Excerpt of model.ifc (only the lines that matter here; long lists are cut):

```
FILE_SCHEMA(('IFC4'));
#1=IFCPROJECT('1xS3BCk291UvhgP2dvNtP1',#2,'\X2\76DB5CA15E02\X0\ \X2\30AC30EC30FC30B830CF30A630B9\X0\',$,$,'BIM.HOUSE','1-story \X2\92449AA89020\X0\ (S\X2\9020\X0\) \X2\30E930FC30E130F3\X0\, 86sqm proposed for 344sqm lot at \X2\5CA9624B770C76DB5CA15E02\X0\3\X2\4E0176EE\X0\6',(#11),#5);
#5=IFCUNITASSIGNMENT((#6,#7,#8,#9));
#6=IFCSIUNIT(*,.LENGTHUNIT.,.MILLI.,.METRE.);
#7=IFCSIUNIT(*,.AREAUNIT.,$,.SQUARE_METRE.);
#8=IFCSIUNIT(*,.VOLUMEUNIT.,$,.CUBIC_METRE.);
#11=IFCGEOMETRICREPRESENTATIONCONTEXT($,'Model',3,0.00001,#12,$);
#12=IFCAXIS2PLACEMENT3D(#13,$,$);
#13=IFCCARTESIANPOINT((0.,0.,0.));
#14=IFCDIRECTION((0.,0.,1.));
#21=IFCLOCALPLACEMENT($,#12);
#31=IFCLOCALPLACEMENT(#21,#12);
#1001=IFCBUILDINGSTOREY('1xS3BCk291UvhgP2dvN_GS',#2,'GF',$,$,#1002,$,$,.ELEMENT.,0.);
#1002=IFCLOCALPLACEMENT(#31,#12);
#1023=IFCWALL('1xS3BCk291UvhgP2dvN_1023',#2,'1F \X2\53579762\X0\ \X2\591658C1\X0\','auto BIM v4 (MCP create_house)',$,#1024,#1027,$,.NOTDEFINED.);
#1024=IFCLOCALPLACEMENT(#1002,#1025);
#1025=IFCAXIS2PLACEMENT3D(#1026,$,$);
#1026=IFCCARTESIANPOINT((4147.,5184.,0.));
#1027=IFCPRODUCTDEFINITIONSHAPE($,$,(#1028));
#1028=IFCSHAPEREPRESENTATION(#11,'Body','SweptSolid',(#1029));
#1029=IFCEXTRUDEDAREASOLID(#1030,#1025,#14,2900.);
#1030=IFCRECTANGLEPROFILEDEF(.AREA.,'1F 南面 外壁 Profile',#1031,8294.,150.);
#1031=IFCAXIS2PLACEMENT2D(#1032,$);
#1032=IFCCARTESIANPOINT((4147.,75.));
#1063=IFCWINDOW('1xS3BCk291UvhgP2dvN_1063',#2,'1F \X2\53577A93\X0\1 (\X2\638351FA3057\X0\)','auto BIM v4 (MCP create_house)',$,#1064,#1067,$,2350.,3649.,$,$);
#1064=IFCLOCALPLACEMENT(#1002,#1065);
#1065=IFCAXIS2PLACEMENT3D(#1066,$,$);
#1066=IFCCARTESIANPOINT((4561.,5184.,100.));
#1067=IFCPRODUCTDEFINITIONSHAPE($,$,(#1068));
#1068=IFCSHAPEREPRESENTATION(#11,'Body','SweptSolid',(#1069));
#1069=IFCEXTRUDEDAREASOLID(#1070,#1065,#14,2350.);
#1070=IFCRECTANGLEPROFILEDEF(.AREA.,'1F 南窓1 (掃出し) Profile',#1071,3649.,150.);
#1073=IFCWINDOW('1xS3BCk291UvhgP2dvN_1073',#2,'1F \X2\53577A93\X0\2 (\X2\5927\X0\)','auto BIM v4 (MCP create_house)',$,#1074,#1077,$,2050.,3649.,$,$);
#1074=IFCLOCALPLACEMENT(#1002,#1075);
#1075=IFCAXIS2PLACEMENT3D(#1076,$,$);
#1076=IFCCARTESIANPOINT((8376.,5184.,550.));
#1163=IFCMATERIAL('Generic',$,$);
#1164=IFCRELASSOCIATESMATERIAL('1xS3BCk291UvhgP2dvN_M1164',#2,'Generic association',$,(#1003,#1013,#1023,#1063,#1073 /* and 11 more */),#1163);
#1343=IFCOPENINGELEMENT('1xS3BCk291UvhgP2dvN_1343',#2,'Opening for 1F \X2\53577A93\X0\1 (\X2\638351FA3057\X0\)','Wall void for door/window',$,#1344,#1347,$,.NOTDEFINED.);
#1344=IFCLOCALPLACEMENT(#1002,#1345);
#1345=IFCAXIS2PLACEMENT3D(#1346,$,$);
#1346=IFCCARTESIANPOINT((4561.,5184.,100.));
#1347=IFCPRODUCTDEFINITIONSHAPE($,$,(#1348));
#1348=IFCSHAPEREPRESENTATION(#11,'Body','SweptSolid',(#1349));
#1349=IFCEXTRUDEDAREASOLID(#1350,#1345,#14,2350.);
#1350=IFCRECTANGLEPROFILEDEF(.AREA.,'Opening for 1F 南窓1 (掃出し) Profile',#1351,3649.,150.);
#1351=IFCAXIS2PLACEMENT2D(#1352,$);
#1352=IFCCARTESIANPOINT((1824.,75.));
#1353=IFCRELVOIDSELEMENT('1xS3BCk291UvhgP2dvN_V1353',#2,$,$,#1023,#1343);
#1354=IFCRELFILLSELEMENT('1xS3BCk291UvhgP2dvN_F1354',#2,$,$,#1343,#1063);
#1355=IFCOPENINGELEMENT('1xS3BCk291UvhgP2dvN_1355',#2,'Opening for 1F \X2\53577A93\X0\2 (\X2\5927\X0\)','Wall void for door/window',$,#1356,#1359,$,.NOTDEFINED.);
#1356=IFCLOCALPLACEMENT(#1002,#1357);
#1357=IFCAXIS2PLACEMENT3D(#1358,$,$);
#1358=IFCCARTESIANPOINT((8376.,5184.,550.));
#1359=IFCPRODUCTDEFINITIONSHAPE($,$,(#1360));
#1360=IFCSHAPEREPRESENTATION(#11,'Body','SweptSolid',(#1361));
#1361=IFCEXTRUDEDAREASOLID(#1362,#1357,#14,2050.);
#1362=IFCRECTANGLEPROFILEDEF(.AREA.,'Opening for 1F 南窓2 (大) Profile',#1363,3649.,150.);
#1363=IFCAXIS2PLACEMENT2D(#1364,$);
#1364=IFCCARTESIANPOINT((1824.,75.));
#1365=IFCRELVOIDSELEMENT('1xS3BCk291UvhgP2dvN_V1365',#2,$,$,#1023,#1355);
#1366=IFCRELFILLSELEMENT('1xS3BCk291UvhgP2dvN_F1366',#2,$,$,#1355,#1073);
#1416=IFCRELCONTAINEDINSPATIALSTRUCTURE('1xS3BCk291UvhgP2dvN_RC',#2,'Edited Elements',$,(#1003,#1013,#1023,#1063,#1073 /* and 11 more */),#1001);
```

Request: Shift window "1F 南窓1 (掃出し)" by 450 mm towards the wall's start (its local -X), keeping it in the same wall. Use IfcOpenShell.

```python
import ifcopenshell
import ifcopenshell.api.geometry
import ifcopenshell.util.placement

model = ifcopenshell.open("model.ifc")

window = model.by_guid("1xS3BCk291UvhgP2dvN_1063")
opening = window.FillsVoids[0].RelatingOpeningElement
wall = opening.VoidsElements[0].RelatingBuildingElement

wall_matrix = ifcopenshell.util.placement.get_local_placement(wall.ObjectPlacement)
shift = wall_matrix[:3, 0] * -450.0
before = ifcopenshell.util.placement.get_local_placement(window.ObjectPlacement)[:3, 3].copy()

# The window is not placed relative to its opening, so move both.
for product in (opening, window):
    matrix = ifcopenshell.util.placement.get_local_placement(product.ObjectPlacement)
    matrix[:3, 3] += shift
    ifcopenshell.api.geometry.edit_object_placement(model, product=product, matrix=matrix, is_si=False)

after = ifcopenshell.util.placement.get_local_placement(window.ObjectPlacement)[:3, 3]
print("window moved by", (after - before).round(3) + 0.0)

model.write("model_edited.ifc")
```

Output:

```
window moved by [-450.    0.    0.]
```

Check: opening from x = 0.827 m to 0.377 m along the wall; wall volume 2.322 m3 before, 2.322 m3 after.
